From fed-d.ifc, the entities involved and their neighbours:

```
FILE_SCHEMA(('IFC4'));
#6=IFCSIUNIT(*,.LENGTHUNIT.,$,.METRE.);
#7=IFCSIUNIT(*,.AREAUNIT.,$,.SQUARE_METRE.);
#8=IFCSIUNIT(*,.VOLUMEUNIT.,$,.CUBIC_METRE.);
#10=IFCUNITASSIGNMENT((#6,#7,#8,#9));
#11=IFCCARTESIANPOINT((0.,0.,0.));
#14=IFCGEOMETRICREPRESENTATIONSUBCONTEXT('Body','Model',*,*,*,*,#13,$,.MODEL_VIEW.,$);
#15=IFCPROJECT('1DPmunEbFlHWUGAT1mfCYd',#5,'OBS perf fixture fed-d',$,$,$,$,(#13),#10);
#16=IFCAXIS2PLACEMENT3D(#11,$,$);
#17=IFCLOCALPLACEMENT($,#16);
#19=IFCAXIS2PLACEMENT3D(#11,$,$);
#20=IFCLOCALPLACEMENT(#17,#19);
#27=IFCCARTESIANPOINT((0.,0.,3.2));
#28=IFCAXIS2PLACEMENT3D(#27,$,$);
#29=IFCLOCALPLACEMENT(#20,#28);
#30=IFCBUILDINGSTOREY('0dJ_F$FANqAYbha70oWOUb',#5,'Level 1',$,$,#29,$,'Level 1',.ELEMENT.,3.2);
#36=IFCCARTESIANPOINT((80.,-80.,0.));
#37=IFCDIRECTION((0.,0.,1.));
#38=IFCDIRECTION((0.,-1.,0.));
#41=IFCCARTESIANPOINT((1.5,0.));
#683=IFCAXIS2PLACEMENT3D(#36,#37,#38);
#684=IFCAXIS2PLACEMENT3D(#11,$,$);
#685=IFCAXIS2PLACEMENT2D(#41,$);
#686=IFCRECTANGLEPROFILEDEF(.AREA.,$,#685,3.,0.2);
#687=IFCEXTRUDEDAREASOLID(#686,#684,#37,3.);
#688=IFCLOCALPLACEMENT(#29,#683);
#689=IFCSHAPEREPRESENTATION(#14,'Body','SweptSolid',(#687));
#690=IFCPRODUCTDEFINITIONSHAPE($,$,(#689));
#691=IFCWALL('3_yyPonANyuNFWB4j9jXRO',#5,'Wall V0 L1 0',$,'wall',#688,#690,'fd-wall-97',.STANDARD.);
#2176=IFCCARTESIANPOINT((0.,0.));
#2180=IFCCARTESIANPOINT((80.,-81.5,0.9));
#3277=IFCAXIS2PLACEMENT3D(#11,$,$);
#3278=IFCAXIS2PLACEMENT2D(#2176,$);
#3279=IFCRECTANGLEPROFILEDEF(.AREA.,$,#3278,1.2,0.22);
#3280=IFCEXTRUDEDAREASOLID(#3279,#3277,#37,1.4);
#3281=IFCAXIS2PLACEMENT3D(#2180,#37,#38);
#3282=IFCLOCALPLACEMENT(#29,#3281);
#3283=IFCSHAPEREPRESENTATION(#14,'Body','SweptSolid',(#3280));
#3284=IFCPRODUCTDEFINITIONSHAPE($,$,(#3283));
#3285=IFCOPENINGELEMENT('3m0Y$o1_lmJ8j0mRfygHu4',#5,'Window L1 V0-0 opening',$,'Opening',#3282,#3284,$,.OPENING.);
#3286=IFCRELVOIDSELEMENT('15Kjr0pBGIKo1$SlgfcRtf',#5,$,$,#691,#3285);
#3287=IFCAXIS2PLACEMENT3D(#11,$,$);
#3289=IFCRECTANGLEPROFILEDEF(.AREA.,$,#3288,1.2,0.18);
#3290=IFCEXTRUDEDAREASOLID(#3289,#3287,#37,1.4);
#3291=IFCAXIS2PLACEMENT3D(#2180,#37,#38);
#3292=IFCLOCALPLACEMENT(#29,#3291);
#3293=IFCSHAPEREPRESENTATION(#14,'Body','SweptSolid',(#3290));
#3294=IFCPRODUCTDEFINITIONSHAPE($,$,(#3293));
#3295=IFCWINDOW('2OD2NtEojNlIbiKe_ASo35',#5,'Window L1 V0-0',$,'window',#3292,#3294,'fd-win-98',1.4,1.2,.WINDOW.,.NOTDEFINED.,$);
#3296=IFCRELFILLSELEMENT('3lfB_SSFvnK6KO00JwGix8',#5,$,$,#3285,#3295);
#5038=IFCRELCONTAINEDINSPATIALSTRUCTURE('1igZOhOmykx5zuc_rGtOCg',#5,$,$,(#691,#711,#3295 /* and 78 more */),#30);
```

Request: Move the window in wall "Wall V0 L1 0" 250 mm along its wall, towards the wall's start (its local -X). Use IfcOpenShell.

```python
import ifcopenshell
import ifcopenshell.api.geometry
import ifcopenshell.util.placement

model = ifcopenshell.open("fed-d.ifc")

window = model.by_guid("2OD2NtEojNlIbiKe_ASo35")
opening = window.FillsVoids[0].RelatingOpeningElement
wall = opening.VoidsElements[0].RelatingBuildingElement

wall_matrix = ifcopenshell.util.placement.get_local_placement(wall.ObjectPlacement)
shift = wall_matrix[:3, 0] * -0.25
before = ifcopenshell.util.placement.get_local_placement(window.ObjectPlacement)[:3, 3].copy()

# The window is not placed relative to its opening, so move both.
for product in (opening, window):
    matrix = ifcopenshell.util.placement.get_local_placement(product.ObjectPlacement)
    matrix[:3, 3] += shift
    ifcopenshell.api.geometry.edit_object_placement(model, product=product, matrix=matrix, is_si=False)

after = ifcopenshell.util.placement.get_local_placement(window.ObjectPlacement)[:3, 3]
print("window moved by", (after - before).round(3) + 0.0)

model.write("fed-d_rev.ifc")
```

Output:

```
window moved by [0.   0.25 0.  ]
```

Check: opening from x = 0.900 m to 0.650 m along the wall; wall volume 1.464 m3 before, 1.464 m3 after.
